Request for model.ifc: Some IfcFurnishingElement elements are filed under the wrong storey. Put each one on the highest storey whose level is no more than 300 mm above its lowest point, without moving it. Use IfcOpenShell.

First a look at what the model holds.

```python
import ifcopenshell
import ifcopenshell.util.element
import ifcopenshell.util.placement

model = ifcopenshell.open("model.ifc")
print(model.schema)
for storey in model.by_type("IfcBuildingStorey"):
    level = ifcopenshell.util.placement.get_storey_elevation(storey)
    count = sum(e.is_a("IfcFurnishingElement") for e in ifcopenshell.util.element.get_contained(storey))
    print(storey.id(), storey.Name, round(level, 3), count, sep=" | ")
```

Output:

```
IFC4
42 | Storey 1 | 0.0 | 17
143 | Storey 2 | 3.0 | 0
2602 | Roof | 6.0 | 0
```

```python
import ifcopenshell
import ifcopenshell.api.spatial
import ifcopenshell.geom
import ifcopenshell.util.element
import ifcopenshell.util.placement
import ifcopenshell.util.shape
import ifcopenshell.util.unit

model = ifcopenshell.open("model.ifc")
unit_scale = ifcopenshell.util.unit.calculate_unit_scale(model)
settings = ifcopenshell.geom.settings()

levels = sorted(
    ((ifcopenshell.util.placement.get_storey_elevation(s) * unit_scale, s) for s in model.by_type("IfcBuildingStorey")),
    key=lambda pair: pair[0],
)

for e in model.by_type("IfcFurnishingElement"):
    current = e.ContainedInStructure[0].RelatingStructure if e.ContainedInStructure else None
    if current is None or not current.is_a("IfcBuildingStorey"):
        continue
    shape = ifcopenshell.geom.create_shape(settings, e)
    bottom = ifcopenshell.util.shape.get_shape_bottom_elevation(shape, shape.geometry)
    below = [s for level, s in levels if level <= bottom + 0.3]
    storey = below[-1] if below else levels[0][1]
    if storey != current:
        # assign_container keeps the world position.
        ifcopenshell.api.spatial.assign_container(model, products=[e], relating_structure=storey)
        print(e.id(), current.Name, "->", storey.Name)

model.write("model_rev.ifc")
```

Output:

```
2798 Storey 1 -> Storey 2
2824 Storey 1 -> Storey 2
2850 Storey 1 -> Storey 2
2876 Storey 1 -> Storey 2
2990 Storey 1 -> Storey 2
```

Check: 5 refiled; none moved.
